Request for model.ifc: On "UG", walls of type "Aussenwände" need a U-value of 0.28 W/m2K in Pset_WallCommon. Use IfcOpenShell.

First a look at what the model holds.

```python
import ifcopenshell
import ifcopenshell.util.element

model = ifcopenshell.open("model.ifc")
print(model.schema)
storey = next(s for s in model.by_type("IfcBuildingStorey") if s.Name == "UG")
walls = [e for e in ifcopenshell.util.element.get_decomposition(storey) if e.is_a("IfcWall")]
seen = {}
for e in walls:
    element_type = ifcopenshell.util.element.get_type(e)
    key = (element_type.Name if element_type != e and element_type else None, ifcopenshell.util.element.get_pset(e, "Pset_WallCommon", "ThermalTransmittance"))
    seen[key] = seen.get(key, 0) + 1
for (name, value), count in sorted(seen.items(), key=str):
    print(count, "x", name, "|", value)
```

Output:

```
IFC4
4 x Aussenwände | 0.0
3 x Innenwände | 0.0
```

```python
import ifcopenshell
import ifcopenshell.api.pset
import ifcopenshell.util.element

model = ifcopenshell.open("model.ifc")

storey = next(s for s in model.by_type("IfcBuildingStorey") if s.Name == "UG")
walls = [e for e in ifcopenshell.util.element.get_decomposition(storey) if e.is_a("IfcWall")]

count = 0
for e in walls:
    element_type = ifcopenshell.util.element.get_type(e)
    if element_type in (None, e) or element_type.Name != "Aussenwände":
        continue
    # add_pset returns the element's existing set when there is one.
    pset = ifcopenshell.api.pset.add_pset(model, product=e, name="Pset_WallCommon")
    ifcopenshell.api.pset.edit_pset(model, pset=pset, properties={"ThermalTransmittance": 0.28})
    count += 1

print(count, "walls updated")

model.write("model-out.ifc")
```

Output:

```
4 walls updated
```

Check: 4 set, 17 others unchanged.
